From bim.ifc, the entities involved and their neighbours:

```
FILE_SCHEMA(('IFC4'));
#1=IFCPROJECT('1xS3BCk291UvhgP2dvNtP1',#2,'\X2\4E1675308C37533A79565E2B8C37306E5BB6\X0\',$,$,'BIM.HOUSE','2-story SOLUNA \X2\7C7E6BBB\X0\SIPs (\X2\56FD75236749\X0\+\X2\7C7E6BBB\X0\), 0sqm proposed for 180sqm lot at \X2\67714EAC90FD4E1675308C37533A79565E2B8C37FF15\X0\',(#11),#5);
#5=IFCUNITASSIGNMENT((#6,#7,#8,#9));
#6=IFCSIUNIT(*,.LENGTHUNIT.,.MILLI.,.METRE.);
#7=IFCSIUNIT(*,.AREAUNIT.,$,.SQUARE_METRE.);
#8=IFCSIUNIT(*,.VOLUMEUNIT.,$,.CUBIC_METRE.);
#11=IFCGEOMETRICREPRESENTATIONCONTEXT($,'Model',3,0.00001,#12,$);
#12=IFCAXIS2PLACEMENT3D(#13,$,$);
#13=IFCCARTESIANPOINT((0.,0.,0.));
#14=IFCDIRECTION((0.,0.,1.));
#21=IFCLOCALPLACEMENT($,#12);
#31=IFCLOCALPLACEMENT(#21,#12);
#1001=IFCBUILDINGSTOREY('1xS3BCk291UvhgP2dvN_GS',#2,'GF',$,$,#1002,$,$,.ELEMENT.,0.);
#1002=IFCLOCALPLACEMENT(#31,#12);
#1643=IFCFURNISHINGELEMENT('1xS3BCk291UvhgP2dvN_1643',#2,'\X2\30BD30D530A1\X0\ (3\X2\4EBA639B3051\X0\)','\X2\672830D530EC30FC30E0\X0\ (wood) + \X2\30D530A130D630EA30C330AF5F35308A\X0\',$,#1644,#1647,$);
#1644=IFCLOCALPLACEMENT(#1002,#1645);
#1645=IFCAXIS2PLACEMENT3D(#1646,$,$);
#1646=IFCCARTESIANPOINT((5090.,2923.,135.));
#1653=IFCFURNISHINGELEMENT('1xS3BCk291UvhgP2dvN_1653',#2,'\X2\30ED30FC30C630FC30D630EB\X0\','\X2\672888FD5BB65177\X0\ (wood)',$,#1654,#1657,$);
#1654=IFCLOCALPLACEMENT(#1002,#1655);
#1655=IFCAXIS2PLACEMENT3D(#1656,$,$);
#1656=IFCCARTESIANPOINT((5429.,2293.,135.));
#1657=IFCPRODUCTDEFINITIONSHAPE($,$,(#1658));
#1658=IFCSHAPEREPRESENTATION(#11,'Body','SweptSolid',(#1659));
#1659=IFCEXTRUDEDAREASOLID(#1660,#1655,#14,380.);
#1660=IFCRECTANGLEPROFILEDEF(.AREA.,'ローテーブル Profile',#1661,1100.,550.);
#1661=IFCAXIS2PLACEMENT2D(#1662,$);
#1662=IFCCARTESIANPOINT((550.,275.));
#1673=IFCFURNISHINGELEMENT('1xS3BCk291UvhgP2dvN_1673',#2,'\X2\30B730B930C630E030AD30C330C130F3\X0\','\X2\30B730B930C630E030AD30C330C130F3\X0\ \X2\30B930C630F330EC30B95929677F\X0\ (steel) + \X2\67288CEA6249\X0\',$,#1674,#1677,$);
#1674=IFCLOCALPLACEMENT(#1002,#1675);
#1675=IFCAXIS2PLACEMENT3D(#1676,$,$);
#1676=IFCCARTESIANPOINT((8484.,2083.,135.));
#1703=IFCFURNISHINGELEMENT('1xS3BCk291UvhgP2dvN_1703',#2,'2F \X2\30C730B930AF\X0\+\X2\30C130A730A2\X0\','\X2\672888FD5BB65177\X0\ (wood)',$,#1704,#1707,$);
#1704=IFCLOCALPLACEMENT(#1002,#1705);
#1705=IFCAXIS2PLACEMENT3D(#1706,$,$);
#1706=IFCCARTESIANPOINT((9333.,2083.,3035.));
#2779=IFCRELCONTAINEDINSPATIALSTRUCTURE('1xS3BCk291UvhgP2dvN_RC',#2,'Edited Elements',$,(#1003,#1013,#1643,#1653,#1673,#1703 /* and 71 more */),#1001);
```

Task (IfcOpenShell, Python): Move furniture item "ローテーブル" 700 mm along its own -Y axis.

```python
import ifcopenshell
import ifcopenshell.api.geometry
import ifcopenshell.util.placement
import ifcopenshell.util.unit

model = ifcopenshell.open("bim.ifc")
unit_scale = ifcopenshell.util.unit.calculate_unit_scale(model)

item = model.by_id(1653)
matrix = ifcopenshell.util.placement.get_local_placement(item.ObjectPlacement)
matrix[:3, 3] -= matrix[:3, 1] * 0.7 / unit_scale
ifcopenshell.api.geometry.edit_object_placement(model, product=item, matrix=matrix, is_si=False)

print(ifcopenshell.util.placement.get_local_placement(item.ObjectPlacement).round(3) + 0.0)

model.write("bim_rev.ifc")
```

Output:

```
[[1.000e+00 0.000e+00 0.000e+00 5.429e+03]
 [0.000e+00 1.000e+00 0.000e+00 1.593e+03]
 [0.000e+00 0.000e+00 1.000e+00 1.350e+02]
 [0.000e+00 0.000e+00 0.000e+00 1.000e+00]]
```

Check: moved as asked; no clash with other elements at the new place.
